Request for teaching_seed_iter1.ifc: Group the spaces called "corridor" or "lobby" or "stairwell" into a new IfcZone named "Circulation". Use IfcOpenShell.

First a look at what the model holds.

```python
import ifcopenshell

model = ifcopenshell.open("teaching_seed_iter1.ifc")
print(model.schema)
seen = {}
for space in model.by_type("IfcSpace"):
    seen[space.LongName] = seen.get(space.LongName, 0) + 1
for name, count in sorted(seen.items(), key=str):
    print(count, "x", name)
print("zones:", [z.Name for z in model.by_type("IfcZone")][:20])
```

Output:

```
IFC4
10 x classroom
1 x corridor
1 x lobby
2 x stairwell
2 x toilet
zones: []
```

```python
import ifcopenshell
import ifcopenshell.api.group
import ifcopenshell.api.root

model = ifcopenshell.open("teaching_seed_iter1.ifc")

names = {"corridor", "lobby", "stairwell"}
spaces = [s for s in model.by_type("IfcSpace") if s.LongName in names]

zone = ifcopenshell.api.root.create_entity(model, ifc_class="IfcZone", name="Circulation")
ifcopenshell.api.group.assign_group(model, products=spaces, group=zone)
print(len(spaces), "spaces in", zone.Name)

model.write("teaching_seed_iter1_edited.ifc")
```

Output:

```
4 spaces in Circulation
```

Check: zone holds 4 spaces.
